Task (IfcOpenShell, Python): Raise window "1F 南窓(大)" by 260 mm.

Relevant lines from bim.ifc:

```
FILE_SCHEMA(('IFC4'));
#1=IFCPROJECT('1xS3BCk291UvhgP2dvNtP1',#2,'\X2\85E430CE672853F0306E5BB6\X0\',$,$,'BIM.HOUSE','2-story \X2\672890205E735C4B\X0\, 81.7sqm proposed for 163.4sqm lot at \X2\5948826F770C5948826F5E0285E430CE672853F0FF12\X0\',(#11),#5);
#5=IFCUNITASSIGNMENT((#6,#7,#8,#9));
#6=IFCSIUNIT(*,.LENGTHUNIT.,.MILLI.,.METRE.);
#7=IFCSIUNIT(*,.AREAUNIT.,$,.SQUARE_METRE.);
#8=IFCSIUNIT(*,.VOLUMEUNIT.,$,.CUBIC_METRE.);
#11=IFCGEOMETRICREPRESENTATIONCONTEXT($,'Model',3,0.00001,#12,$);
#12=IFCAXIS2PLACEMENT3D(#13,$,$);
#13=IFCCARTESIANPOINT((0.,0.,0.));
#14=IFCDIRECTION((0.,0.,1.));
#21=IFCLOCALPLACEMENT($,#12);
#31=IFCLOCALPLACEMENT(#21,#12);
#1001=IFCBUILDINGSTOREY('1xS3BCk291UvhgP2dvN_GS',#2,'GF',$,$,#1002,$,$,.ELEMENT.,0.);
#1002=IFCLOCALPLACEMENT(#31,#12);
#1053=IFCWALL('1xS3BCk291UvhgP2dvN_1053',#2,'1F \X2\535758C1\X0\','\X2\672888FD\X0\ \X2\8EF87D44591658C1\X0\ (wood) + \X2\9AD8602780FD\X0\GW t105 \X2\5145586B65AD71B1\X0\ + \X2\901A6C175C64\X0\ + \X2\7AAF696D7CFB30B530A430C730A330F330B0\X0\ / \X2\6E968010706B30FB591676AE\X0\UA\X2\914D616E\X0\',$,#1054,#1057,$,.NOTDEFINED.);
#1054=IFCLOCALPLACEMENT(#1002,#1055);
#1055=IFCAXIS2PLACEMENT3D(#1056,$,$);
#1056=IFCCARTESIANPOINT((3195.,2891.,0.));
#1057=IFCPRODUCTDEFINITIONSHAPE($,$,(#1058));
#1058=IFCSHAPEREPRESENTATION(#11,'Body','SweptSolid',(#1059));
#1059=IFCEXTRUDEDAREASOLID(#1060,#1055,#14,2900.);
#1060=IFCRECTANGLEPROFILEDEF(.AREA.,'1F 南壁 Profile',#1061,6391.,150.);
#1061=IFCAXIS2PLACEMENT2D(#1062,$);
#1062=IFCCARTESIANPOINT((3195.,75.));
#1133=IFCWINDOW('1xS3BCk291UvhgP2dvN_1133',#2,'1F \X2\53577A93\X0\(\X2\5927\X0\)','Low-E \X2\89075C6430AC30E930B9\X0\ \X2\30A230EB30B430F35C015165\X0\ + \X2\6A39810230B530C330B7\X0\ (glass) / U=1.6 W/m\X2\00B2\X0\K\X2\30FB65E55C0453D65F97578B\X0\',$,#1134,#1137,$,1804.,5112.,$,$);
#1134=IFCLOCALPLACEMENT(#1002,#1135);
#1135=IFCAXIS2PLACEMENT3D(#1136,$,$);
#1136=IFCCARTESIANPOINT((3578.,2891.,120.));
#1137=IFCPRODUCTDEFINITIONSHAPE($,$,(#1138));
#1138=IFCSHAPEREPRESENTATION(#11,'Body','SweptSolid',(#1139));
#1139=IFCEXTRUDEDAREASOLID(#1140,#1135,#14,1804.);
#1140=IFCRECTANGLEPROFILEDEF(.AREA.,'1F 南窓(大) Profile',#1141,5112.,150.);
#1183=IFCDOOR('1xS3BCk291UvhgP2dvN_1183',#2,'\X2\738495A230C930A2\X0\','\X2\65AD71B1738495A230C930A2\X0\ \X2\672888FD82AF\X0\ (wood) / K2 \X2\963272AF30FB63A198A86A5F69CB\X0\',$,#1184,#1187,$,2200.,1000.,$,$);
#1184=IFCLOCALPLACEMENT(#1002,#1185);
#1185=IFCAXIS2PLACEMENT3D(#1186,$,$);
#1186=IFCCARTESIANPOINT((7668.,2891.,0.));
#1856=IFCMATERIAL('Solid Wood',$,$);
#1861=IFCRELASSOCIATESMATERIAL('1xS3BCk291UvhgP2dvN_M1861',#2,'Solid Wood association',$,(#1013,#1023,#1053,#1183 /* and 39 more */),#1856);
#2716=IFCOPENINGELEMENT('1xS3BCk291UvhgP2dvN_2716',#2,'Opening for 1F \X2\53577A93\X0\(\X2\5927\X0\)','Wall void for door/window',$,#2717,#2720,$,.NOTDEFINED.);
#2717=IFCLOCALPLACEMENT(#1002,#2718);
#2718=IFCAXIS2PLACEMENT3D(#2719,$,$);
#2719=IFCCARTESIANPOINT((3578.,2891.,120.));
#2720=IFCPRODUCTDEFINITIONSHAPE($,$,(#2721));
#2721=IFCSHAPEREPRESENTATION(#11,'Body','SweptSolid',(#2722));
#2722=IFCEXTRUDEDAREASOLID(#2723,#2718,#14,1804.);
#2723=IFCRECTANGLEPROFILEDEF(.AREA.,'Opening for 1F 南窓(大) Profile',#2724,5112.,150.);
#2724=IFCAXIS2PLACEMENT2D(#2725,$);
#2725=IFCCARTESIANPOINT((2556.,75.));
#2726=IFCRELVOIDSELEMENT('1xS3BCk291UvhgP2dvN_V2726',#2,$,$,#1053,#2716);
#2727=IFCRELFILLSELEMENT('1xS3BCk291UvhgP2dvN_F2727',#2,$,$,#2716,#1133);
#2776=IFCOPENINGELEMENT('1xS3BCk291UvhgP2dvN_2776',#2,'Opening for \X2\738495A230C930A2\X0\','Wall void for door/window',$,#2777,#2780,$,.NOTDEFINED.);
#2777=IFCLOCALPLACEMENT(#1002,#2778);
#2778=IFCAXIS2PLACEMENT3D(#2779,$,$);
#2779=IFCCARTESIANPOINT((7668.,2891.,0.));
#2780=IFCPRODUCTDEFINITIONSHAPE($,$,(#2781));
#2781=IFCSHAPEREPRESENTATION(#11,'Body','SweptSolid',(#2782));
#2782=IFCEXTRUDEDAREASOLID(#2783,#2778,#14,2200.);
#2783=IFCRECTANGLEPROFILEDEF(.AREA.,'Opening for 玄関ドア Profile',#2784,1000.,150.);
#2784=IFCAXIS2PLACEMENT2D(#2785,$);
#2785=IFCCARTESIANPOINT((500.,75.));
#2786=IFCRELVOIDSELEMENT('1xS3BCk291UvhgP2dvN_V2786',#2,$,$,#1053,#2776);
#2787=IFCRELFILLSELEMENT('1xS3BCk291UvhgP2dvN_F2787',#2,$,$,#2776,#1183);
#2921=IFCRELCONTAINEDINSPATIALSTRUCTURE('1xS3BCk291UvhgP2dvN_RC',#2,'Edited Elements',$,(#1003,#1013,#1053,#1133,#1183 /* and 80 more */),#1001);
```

```python
import numpy as np
import ifcopenshell
import ifcopenshell.api.geometry
import ifcopenshell.util.placement
import ifcopenshell.util.unit

model = ifcopenshell.open("bim.ifc")
unit_scale = ifcopenshell.util.unit.calculate_unit_scale(model)

window = model.by_guid("1xS3BCk291UvhgP2dvN_1133")
opening = window.FillsVoids[0].RelatingOpeningElement
dz = 0.26 / unit_scale

shift = np.array([0.0, 0.0, dz])
# The window is not placed relative to its opening, so move both.
for product in (opening, window):
    matrix = ifcopenshell.util.placement.get_local_placement(product.ObjectPlacement)
    matrix[:3, 3] += shift
    ifcopenshell.api.geometry.edit_object_placement(model, product=product, matrix=matrix, is_si=False)

print(f"moved by {dz * unit_scale:+.3f} m")

model.write("bim_v2.ifc")
```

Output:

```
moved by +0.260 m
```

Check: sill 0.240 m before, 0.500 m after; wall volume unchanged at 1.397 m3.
